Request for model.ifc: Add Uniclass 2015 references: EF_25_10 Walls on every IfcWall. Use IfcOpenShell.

First a look at what the model holds.

```python
import ifcopenshell

model = ifcopenshell.open("model.ifc")
print(model.schema)
print("classifications:", [c.Name for c in model.by_type("IfcClassification")])
for ifc_class in ("IfcDoor", "IfcRoof", "IfcStair", "IfcWall", "IfcWindow"):
    print(ifc_class, len(model.by_type(ifc_class)))
```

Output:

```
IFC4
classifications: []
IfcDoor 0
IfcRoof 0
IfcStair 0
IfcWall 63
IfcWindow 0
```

```python
import ifcopenshell
import ifcopenshell.api.classification

model = ifcopenshell.open("model.ifc")

system = ifcopenshell.api.classification.add_classification(model, classification="Uniclass 2015")

codes = {
    "IfcWall": ("EF_25_10", "Walls"),
}
for ifc_class, (code, name) in codes.items():
    products = model.by_type(ifc_class)
    ifcopenshell.api.classification.add_reference(
        model, products=products, classification=system, identification=code, name=name
    )
    print(code, len(products))

model.write("model_updated.ifc")
```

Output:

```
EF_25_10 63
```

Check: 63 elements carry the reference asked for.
